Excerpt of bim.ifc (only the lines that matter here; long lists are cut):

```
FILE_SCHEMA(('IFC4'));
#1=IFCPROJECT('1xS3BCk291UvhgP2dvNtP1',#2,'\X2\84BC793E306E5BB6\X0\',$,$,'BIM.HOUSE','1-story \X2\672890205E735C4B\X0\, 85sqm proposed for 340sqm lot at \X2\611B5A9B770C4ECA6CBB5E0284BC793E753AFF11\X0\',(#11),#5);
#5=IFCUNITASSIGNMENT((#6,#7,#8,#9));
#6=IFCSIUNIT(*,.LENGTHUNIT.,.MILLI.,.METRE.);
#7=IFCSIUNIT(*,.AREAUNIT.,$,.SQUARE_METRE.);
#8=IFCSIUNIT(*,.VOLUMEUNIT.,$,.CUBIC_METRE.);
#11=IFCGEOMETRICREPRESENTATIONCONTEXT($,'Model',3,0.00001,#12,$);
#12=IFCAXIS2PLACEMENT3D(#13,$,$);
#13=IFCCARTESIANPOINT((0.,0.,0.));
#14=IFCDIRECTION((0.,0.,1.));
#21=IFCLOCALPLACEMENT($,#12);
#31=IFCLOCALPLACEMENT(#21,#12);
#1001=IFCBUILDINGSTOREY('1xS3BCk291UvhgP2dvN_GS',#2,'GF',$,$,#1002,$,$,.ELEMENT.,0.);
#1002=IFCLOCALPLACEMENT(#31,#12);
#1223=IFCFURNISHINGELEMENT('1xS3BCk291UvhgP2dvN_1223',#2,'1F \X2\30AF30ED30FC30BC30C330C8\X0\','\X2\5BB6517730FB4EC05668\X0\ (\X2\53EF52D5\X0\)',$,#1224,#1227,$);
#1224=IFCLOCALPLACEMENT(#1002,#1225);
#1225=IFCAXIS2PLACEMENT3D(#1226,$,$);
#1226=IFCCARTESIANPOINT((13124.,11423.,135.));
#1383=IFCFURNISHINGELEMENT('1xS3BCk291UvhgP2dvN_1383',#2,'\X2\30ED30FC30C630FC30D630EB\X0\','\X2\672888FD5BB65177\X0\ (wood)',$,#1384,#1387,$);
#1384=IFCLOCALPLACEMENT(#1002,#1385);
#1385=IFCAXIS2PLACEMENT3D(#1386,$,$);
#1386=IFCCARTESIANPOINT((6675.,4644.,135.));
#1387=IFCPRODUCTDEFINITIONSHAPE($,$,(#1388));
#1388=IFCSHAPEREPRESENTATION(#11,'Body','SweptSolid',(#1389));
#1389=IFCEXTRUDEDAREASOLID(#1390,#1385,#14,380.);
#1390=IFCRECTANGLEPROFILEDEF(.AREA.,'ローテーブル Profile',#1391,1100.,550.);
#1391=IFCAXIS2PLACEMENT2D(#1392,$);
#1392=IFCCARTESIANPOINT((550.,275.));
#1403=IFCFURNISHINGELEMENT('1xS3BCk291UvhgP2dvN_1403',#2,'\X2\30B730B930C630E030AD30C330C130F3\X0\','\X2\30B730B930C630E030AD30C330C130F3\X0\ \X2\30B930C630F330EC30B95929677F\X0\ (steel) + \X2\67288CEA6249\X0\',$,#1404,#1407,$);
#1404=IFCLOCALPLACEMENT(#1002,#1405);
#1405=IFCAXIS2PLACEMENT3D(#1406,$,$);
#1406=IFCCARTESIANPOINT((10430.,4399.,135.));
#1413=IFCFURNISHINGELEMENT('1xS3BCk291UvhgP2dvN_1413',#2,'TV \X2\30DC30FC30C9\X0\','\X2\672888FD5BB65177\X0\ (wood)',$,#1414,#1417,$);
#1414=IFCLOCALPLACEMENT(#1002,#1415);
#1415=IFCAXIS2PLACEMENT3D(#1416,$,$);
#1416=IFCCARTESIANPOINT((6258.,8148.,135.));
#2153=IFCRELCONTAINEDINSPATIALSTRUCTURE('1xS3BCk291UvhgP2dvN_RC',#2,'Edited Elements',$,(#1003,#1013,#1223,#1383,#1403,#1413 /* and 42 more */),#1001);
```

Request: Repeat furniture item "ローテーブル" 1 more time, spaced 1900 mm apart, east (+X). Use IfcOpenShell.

```python
import numpy as np
import ifcopenshell
import ifcopenshell.api.geometry
import ifcopenshell.api.root
import ifcopenshell.util.element
import ifcopenshell.util.placement

model = ifcopenshell.open("bim.ifc")


def reuse_history(source, copy):
    """copy_class also copies each property set's owner history, people and application; keep the originals."""
    for rel in copy.IsDefinedBy:
        if rel.is_a("IfcRelDefinesByProperties") and (history := rel.RelatingPropertyDefinition.OwnerHistory):
            rel.RelatingPropertyDefinition.OwnerHistory = source.OwnerHistory
            ifcopenshell.util.element.remove_deep2(model, history)


source = model.by_id(1383)
base = ifcopenshell.util.placement.get_local_placement(source.ObjectPlacement)
step = np.array([1.0, 0.0, 0.0]) * 1900.0

for i in range(1, 2):
    copy = ifcopenshell.api.root.copy_class(model, product=source)
    copy.Representation = ifcopenshell.util.element.copy_deep(
        model, source.Representation, exclude=["IfcGeometricRepresentationContext", "IfcRepresentationMap"]
    )
    reuse_history(source, copy)
    matrix = base.copy()
    matrix[:3, 3] += i * step
    print("added at", matrix[:3, 3].round(3) + 0.0)
    ifcopenshell.api.geometry.edit_object_placement(model, product=copy, matrix=matrix, is_si=False)

model.write("bim_edited.ifc")
```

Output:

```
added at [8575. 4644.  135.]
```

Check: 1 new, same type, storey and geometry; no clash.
